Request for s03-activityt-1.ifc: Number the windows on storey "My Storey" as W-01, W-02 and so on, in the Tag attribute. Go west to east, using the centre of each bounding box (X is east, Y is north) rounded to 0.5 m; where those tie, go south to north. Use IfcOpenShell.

First a look at what the model holds.

```python
import ifcopenshell
import ifcopenshell.util.element
import ifcopenshell.util.placement

model = ifcopenshell.open("s03-activityt-1.ifc")
print(model.schema)
storey = next(s for s in model.by_type("IfcBuildingStorey") if s.Name == "My Storey")
windows = [e for e in ifcopenshell.util.element.get_decomposition(storey) if e.is_a("IfcWindow")]
for e in sorted(windows, key=lambda e: e.id()):
    origin = ifcopenshell.util.placement.get_local_placement(e.ObjectPlacement)[:3, 3]
    print(e.id(), e.Tag, e.Name, origin.round(2) + 0.0, sep=" | ")
```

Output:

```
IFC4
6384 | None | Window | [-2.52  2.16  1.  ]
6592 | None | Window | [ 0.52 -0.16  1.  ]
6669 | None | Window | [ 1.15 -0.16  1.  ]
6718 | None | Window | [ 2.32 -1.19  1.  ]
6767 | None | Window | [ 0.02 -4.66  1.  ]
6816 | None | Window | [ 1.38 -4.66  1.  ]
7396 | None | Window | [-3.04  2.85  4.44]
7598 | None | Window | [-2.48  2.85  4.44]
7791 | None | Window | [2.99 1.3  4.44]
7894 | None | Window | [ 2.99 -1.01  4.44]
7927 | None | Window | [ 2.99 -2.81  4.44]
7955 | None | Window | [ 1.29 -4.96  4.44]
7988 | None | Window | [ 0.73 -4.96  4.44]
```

```python
import ifcopenshell
import ifcopenshell.geom
import ifcopenshell.util.element
import ifcopenshell.util.shape

model = ifcopenshell.open("s03-activityt-1.ifc")
settings = ifcopenshell.geom.settings()
settings.set("use-world-coords", True)


def centre(element):
    shape = ifcopenshell.geom.create_shape(settings, element)
    return ifcopenshell.util.shape.get_bbox_centroid(shape.geometry)


storey = next(s for s in model.by_type("IfcBuildingStorey") if s.Name == "My Storey")
windows = [e for e in ifcopenshell.util.element.get_decomposition(storey) if e.is_a("IfcWindow")]

# Insertion points can sit at a corner or the storey origin, so sort by the geometry (in metres).
centres = {e: centre(e) for e in windows}
windows.sort(key=lambda e: (round(centres[e][0] / 0.5), centres[e][1]))

for i, e in enumerate(windows, start=1):
    number = f"W-{i:02d}"
    e.Tag = number
    print(e.id(), number)

model.write("s03-activityt-1_rev.ifc")
```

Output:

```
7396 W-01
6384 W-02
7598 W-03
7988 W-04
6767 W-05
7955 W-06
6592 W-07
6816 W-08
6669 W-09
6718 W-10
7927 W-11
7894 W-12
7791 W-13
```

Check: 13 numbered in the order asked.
